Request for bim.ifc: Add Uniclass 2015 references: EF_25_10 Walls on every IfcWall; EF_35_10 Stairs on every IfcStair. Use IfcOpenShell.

First a look at what the model holds.

```python
import ifcopenshell

model = ifcopenshell.open("bim.ifc")
print(model.schema)
print("classifications:", [c.Name for c in model.by_type("IfcClassification")])
for ifc_class in ("IfcDoor", "IfcRoof", "IfcStair", "IfcWall", "IfcWindow"):
    print(ifc_class, len(model.by_type(ifc_class)))
```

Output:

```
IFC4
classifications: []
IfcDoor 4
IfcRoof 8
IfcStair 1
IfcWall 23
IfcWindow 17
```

```python
import ifcopenshell
import ifcopenshell.api.classification

model = ifcopenshell.open("bim.ifc")

system = ifcopenshell.api.classification.add_classification(model, classification="Uniclass 2015")

codes = {
    "IfcWall": ("EF_25_10", "Walls"),
    "IfcStair": ("EF_35_10", "Stairs"),
}
for ifc_class, (code, name) in codes.items():
    products = model.by_type(ifc_class)
    ifcopenshell.api.classification.add_reference(
        model, products=products, classification=system, identification=code, name=name
    )
    print(code, len(products))

model.write("bim-out.ifc")
```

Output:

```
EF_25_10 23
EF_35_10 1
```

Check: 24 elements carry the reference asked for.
